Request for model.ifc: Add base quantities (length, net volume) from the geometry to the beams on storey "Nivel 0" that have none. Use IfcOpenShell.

First a look at what the model holds.

```python
import ifcopenshell
import ifcopenshell.util.element
import ifcopenshell.util.unit

model = ifcopenshell.open("model.ifc")
print(model.schema)
for unit_type in ("LENGTHUNIT", "AREAUNIT", "VOLUMEUNIT"):
    print(unit_type, ifcopenshell.util.unit.calculate_unit_scale(model, unit_type))
storey = next(s for s in model.by_type("IfcBuildingStorey") if s.Name == "Nivel 0")
beams = [e for e in ifcopenshell.util.element.get_decomposition(storey) if e.is_a("IfcBeam")]
for e in sorted(beams, key=lambda e: e.id()):
    print(e.id(), e.is_a(), e.Name, list(ifcopenshell.util.element.get_psets(e, qtos_only=True)), sep=" | ")
```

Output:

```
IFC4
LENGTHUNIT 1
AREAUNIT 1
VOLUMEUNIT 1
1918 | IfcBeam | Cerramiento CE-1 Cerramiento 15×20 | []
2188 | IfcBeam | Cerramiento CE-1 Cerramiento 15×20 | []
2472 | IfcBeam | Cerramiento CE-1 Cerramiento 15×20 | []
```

```python
import ifcopenshell
import ifcopenshell.api.pset
import ifcopenshell.geom
import ifcopenshell.util.element
import ifcopenshell.util.shape
import ifcopenshell.util.unit

model = ifcopenshell.open("model.ifc")
unit_scale = ifcopenshell.util.unit.calculate_unit_scale(model)
volume_scale = ifcopenshell.util.unit.calculate_unit_scale(model, "VOLUMEUNIT")
settings = ifcopenshell.geom.settings()

storey = next(s for s in model.by_type("IfcBuildingStorey") if s.Name == "Nivel 0")
beams = [e for e in ifcopenshell.util.element.get_decomposition(storey) if e.is_a("IfcBeam")]

for e in sorted(beams, key=lambda e: e.id()):
    if ifcopenshell.util.element.get_psets(e, qtos_only=True, should_inherit=False):
        continue
    # Geometry comes back in metres, in the element's own axes.
    shape = ifcopenshell.geom.create_shape(settings, e)
    values = {
        "Length": ifcopenshell.util.shape.get_max_xyz(shape.geometry) / unit_scale,
        "NetVolume": ifcopenshell.util.shape.get_volume(shape.geometry) / volume_scale,
    }
    qto = ifcopenshell.api.pset.add_qto(model, product=e, name="Qto_BeamBaseQuantities")
    ifcopenshell.api.pset.edit_qto(model, qto=qto, properties=values)
    print(e.id(), {k: round(v, 3) for k, v in values.items()})

model.write("model_rev.ifc")
```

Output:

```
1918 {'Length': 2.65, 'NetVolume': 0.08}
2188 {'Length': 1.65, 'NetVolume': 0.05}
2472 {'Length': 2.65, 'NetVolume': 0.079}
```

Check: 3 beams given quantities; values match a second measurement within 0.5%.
